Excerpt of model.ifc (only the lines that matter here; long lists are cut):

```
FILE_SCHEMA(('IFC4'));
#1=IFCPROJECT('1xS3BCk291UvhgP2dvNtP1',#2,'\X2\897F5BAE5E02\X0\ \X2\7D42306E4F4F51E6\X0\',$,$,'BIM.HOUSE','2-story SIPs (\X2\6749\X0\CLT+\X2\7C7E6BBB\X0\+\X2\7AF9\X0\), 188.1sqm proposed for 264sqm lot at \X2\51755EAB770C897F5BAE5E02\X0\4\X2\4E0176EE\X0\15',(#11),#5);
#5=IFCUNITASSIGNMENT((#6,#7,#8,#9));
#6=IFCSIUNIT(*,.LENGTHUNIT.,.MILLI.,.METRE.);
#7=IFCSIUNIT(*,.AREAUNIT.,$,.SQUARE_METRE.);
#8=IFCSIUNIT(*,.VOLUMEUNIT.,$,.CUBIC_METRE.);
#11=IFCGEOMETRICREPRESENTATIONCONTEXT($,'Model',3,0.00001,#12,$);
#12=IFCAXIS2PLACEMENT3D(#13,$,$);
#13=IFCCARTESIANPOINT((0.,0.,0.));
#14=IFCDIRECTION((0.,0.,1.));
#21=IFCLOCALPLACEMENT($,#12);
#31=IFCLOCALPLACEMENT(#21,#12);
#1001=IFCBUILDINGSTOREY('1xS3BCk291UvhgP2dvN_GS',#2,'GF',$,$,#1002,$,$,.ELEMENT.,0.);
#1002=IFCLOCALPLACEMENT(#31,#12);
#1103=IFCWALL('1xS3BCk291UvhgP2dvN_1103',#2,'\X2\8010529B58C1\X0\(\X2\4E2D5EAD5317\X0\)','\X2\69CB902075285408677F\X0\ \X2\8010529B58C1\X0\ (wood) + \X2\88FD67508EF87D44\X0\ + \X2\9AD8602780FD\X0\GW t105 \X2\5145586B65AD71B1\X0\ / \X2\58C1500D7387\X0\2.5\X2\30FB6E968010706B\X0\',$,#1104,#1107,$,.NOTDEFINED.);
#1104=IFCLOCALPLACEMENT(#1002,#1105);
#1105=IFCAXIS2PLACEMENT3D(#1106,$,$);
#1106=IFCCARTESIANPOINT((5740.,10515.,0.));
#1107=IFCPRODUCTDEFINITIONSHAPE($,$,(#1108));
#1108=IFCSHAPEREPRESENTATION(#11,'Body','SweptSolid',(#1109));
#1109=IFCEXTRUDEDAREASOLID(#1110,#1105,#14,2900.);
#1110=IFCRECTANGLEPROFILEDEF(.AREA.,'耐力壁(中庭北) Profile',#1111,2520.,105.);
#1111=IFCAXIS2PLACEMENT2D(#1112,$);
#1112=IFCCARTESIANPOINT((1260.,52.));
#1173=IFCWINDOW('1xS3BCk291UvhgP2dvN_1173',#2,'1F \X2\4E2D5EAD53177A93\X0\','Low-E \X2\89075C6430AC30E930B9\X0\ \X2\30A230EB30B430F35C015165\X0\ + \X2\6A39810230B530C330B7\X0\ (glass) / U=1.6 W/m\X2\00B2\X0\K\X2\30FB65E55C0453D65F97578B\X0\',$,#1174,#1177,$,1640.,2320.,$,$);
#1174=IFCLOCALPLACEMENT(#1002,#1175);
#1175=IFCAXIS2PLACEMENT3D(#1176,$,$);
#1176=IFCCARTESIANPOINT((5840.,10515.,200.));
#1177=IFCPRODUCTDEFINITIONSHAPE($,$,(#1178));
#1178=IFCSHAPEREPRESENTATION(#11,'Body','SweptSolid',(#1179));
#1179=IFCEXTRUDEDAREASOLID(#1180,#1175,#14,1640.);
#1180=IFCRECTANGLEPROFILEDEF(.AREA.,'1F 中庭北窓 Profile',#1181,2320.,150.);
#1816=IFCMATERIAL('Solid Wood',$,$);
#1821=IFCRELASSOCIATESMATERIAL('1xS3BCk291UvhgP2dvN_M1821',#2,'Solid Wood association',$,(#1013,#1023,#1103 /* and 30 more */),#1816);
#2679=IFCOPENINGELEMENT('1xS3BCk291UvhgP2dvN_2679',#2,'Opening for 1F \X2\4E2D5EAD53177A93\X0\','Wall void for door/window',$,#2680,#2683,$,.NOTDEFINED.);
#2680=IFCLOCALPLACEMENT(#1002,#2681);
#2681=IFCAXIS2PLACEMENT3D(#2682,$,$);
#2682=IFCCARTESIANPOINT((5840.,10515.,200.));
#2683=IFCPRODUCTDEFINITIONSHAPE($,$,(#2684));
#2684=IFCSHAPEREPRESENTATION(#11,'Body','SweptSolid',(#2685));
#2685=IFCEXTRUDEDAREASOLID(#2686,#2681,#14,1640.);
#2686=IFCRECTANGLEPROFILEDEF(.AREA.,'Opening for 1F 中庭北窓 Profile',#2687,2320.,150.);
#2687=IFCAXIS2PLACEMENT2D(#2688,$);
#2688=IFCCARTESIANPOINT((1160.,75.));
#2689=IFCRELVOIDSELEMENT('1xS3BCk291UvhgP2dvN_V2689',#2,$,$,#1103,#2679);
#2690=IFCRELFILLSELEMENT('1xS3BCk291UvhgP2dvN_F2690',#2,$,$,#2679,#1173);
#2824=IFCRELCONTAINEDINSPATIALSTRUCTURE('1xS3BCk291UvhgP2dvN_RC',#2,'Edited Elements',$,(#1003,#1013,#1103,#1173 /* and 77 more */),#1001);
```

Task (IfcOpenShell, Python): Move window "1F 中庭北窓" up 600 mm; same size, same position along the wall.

```python
import numpy as np
import ifcopenshell
import ifcopenshell.api.geometry
import ifcopenshell.util.placement
import ifcopenshell.util.unit

model = ifcopenshell.open("model.ifc")
unit_scale = ifcopenshell.util.unit.calculate_unit_scale(model)

window = model.by_guid("1xS3BCk291UvhgP2dvN_1173")
opening = window.FillsVoids[0].RelatingOpeningElement
dz = 600.0

shift = np.array([0.0, 0.0, dz])
# The window is not placed relative to its opening, so move both.
for product in (opening, window):
    matrix = ifcopenshell.util.placement.get_local_placement(product.ObjectPlacement)
    matrix[:3, 3] += shift
    ifcopenshell.api.geometry.edit_object_placement(model, product=product, matrix=matrix, is_si=False)

print(f"moved by {dz * unit_scale:+.3f} m")

model.write("model_v2.ifc")
```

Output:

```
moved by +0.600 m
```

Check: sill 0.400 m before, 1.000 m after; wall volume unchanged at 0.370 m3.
